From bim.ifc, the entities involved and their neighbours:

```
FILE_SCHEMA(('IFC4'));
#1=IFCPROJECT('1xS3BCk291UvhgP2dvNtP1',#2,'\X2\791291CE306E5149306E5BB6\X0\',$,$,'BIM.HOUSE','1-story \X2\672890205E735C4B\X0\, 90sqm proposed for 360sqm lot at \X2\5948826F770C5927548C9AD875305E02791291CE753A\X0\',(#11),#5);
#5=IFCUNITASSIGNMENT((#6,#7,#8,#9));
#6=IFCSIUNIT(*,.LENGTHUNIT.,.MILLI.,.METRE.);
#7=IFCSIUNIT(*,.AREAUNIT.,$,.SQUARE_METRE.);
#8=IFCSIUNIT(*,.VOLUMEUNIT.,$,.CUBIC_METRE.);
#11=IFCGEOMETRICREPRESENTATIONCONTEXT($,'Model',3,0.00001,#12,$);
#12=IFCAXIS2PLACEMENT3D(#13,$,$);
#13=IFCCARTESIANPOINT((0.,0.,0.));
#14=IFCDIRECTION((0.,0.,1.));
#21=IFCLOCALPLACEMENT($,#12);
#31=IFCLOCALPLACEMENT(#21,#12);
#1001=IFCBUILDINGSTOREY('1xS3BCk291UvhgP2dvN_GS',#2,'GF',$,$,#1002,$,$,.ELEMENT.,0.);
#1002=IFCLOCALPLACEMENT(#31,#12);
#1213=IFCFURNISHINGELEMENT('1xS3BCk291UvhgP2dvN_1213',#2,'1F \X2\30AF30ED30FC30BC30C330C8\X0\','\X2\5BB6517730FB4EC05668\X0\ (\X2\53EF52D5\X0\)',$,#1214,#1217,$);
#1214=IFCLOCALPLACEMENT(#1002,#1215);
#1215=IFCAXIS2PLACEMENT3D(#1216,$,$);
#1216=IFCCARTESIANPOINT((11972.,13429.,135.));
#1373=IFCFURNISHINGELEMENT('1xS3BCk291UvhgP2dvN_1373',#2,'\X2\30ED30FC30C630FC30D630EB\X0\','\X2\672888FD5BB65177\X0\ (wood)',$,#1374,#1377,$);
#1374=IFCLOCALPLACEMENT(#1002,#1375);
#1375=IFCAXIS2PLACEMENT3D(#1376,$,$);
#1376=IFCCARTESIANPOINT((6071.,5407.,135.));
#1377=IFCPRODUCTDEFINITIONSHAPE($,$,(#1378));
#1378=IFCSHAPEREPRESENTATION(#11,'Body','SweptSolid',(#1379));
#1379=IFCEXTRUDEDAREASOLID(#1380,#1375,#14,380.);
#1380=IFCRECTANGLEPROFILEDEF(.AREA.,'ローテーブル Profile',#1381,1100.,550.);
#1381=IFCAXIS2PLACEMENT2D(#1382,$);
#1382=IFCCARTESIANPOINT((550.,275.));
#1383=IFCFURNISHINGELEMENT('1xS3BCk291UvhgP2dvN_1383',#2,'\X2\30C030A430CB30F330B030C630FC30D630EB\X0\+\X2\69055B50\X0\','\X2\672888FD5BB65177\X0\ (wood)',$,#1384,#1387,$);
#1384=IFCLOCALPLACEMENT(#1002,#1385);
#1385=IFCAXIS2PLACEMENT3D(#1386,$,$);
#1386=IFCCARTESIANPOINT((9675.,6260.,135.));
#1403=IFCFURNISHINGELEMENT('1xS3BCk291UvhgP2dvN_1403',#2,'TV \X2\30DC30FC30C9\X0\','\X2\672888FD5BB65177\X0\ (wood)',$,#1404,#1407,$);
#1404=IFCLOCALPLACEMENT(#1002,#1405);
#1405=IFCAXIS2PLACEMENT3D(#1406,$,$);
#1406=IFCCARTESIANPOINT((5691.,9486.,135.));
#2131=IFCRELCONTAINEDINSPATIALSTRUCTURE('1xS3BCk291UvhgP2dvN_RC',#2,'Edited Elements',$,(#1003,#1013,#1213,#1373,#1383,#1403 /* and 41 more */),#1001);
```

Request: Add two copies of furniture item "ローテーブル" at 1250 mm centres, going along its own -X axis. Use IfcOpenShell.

```python
import ifcopenshell
import ifcopenshell.api.geometry
import ifcopenshell.api.root
import ifcopenshell.util.element
import ifcopenshell.util.placement

model = ifcopenshell.open("bim.ifc")


def reuse_history(source, copy):
    """copy_class also copies each property set's owner history, people and application; keep the originals."""
    for rel in copy.IsDefinedBy:
        if rel.is_a("IfcRelDefinesByProperties") and (history := rel.RelatingPropertyDefinition.OwnerHistory):
            rel.RelatingPropertyDefinition.OwnerHistory = source.OwnerHistory
            ifcopenshell.util.element.remove_deep2(model, history)


source = model.by_guid("1xS3BCk291UvhgP2dvN_1373")
base = ifcopenshell.util.placement.get_local_placement(source.ObjectPlacement)
step = -base[:3, 0] * 1250.0

for i in range(1, 3):
    copy = ifcopenshell.api.root.copy_class(model, product=source)
    copy.Representation = ifcopenshell.util.element.copy_deep(
        model, source.Representation, exclude=["IfcGeometricRepresentationContext", "IfcRepresentationMap"]
    )
    reuse_history(source, copy)
    matrix = base.copy()
    matrix[:3, 3] += i * step
    print("added at", matrix[:3, 3].round(3) + 0.0)
    ifcopenshell.api.geometry.edit_object_placement(model, product=copy, matrix=matrix, is_si=False)

model.write("bim_v2.ifc")
```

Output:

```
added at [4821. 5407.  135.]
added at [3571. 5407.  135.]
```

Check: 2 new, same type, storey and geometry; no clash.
